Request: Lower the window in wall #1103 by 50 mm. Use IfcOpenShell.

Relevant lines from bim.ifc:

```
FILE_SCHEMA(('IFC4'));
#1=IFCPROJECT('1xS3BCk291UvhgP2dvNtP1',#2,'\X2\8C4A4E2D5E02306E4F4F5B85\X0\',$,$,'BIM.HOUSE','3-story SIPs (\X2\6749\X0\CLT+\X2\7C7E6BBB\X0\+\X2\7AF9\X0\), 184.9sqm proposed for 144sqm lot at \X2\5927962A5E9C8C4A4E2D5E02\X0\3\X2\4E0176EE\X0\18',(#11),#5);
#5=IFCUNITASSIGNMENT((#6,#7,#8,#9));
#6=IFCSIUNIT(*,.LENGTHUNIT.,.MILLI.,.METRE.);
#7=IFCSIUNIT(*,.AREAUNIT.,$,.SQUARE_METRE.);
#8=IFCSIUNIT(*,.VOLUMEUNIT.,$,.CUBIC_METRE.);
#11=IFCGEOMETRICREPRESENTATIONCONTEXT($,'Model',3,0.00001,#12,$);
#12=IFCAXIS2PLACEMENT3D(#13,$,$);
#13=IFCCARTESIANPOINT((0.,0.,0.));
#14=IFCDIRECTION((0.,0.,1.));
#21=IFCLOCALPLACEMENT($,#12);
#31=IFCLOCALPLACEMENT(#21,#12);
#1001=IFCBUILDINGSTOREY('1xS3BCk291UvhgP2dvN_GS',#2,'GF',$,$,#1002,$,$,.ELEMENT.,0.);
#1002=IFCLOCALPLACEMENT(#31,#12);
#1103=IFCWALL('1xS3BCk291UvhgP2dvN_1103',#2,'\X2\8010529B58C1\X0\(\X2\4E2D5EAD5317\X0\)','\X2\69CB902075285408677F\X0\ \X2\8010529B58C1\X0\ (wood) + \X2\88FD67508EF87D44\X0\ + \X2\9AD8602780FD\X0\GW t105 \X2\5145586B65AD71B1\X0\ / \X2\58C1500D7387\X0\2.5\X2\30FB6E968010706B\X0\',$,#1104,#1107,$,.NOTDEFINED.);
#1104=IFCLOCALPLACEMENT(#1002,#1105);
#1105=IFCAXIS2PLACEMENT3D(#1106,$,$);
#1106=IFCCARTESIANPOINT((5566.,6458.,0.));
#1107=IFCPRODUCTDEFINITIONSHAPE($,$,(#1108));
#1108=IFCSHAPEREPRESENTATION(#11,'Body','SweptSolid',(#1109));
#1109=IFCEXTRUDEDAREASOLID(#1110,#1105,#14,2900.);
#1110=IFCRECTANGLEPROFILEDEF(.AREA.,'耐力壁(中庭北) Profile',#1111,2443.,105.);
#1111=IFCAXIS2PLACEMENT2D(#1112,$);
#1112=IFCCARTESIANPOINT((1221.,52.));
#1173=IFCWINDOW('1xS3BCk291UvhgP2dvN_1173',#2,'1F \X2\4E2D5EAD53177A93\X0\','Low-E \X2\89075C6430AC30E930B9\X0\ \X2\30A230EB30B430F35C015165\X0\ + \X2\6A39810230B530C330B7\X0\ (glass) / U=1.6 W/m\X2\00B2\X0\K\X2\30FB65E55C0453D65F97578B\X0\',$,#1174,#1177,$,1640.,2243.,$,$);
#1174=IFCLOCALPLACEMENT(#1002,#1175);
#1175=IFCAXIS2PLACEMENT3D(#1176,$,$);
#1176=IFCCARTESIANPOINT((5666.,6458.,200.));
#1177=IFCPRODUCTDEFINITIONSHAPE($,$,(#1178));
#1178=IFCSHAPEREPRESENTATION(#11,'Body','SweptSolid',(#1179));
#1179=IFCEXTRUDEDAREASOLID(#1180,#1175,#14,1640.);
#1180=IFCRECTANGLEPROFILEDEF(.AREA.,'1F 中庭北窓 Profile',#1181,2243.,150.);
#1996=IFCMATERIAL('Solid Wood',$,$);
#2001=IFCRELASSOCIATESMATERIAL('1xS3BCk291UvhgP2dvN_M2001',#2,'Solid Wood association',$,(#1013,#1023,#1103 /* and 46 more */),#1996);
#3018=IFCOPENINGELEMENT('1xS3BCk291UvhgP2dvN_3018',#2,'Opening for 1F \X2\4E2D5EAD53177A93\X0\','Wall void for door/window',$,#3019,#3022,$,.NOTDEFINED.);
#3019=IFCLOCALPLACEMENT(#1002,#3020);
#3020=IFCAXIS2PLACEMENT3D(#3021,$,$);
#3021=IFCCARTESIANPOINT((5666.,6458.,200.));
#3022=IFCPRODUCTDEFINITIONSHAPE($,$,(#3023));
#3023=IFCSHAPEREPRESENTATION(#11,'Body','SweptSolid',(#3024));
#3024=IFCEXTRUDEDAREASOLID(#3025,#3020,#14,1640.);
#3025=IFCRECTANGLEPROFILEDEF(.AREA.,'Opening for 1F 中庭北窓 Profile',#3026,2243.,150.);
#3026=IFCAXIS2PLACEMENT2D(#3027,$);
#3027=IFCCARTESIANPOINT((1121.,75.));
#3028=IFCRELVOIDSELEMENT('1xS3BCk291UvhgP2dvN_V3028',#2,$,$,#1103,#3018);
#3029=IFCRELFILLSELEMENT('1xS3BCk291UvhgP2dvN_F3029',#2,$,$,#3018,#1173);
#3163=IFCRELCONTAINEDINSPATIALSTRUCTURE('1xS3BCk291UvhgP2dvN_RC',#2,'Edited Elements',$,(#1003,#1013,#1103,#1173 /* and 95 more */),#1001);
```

```python
import numpy as np
import ifcopenshell
import ifcopenshell.api.geometry
import ifcopenshell.util.placement
import ifcopenshell.util.unit

model = ifcopenshell.open("bim.ifc")
unit_scale = ifcopenshell.util.unit.calculate_unit_scale(model)

window = model.by_id(1173)
opening = window.FillsVoids[0].RelatingOpeningElement
dz = -50.0

shift = np.array([0.0, 0.0, dz])
# The window is not placed relative to its opening, so move both.
for product in (opening, window):
    matrix = ifcopenshell.util.placement.get_local_placement(product.ObjectPlacement)
    matrix[:3, 3] += shift
    ifcopenshell.api.geometry.edit_object_placement(model, product=product, matrix=matrix, is_si=False)

print(f"moved by {dz * unit_scale:+.3f} m")

model.write("bim_edited.ifc")
```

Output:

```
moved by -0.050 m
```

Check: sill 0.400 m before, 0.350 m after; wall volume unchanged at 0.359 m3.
